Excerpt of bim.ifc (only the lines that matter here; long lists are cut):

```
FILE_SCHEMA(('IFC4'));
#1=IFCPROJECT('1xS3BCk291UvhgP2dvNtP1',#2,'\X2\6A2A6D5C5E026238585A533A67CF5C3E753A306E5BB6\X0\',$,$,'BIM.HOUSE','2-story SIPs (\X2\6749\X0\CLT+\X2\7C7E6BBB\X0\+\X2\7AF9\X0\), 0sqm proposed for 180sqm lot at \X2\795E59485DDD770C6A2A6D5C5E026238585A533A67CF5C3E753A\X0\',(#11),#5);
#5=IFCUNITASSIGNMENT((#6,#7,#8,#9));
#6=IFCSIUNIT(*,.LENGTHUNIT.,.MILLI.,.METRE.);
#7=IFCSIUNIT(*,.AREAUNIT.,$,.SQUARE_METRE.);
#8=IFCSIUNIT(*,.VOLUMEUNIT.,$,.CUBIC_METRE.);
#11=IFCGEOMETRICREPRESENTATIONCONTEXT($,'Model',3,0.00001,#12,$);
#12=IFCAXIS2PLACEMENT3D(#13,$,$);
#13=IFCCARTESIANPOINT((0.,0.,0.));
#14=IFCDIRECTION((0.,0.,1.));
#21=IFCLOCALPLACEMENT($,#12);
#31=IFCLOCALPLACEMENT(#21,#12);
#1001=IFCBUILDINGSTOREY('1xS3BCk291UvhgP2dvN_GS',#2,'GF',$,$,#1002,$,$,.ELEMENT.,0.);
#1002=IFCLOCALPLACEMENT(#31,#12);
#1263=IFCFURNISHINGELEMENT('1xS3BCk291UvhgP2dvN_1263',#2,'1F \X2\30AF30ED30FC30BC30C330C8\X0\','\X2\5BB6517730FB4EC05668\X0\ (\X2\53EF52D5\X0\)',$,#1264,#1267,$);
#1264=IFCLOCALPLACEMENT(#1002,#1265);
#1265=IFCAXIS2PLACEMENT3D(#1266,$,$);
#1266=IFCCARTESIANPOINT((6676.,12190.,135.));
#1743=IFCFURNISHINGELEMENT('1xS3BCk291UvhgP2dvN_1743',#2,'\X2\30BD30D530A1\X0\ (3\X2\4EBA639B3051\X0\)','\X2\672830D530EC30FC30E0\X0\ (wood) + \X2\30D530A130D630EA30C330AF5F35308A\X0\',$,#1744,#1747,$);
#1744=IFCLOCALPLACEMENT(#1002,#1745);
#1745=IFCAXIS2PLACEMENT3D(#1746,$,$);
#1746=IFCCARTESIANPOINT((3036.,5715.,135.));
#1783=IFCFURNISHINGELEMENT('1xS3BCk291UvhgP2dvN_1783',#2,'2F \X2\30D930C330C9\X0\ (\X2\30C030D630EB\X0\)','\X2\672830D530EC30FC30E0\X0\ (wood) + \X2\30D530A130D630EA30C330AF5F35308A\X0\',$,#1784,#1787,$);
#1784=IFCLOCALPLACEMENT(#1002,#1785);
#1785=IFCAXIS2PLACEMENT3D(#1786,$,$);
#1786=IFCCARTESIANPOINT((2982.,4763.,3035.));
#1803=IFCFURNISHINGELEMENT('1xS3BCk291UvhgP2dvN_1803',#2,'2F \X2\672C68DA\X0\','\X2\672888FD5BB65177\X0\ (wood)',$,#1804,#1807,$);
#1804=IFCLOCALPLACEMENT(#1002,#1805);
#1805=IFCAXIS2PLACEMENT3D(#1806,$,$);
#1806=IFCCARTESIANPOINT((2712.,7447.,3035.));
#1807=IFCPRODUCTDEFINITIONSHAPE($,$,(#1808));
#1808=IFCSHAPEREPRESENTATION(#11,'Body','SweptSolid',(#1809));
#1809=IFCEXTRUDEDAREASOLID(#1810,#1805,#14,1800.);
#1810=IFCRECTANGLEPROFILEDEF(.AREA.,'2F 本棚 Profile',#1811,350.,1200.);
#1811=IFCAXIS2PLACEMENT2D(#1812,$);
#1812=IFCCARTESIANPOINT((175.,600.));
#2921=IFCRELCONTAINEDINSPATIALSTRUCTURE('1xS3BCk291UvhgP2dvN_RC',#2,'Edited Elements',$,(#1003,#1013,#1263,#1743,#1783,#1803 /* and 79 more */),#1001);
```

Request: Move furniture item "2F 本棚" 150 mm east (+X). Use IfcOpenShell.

```python
import ifcopenshell
import ifcopenshell.api.geometry
import ifcopenshell.util.placement
import ifcopenshell.util.unit

model = ifcopenshell.open("bim.ifc")
unit_scale = ifcopenshell.util.unit.calculate_unit_scale(model)

item = model.by_guid("1xS3BCk291UvhgP2dvN_1803")
matrix = ifcopenshell.util.placement.get_local_placement(item.ObjectPlacement)
matrix[0, 3] += 0.15 / unit_scale
ifcopenshell.api.geometry.edit_object_placement(model, product=item, matrix=matrix, is_si=False)

print(ifcopenshell.util.placement.get_local_placement(item.ObjectPlacement).round(3) + 0.0)

model.write("bim_updated.ifc")
```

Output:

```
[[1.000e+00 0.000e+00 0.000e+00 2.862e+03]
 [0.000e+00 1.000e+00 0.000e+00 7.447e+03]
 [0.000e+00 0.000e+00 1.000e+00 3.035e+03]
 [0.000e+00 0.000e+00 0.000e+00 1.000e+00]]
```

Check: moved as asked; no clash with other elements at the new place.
